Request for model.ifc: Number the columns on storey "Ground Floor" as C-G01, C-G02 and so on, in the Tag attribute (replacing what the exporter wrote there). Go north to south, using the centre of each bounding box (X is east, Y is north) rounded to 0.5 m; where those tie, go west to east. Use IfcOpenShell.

First a look at what the model holds.

```python
import ifcopenshell
import ifcopenshell.util.element
import ifcopenshell.util.placement

model = ifcopenshell.open("model.ifc")
print(model.schema)
storey = next(s for s in model.by_type("IfcBuildingStorey") if s.Name == "Ground Floor")
columns = [e for e in ifcopenshell.util.element.get_decomposition(storey) if e.is_a("IfcColumn")]
for e in sorted(columns, key=lambda e: e.id()):
    origin = ifcopenshell.util.placement.get_local_placement(e.ObjectPlacement)[:3, 3]
    print(e.id(), e.Tag, e.Name, origin.round(2) + 0.0, sep=" | ")
```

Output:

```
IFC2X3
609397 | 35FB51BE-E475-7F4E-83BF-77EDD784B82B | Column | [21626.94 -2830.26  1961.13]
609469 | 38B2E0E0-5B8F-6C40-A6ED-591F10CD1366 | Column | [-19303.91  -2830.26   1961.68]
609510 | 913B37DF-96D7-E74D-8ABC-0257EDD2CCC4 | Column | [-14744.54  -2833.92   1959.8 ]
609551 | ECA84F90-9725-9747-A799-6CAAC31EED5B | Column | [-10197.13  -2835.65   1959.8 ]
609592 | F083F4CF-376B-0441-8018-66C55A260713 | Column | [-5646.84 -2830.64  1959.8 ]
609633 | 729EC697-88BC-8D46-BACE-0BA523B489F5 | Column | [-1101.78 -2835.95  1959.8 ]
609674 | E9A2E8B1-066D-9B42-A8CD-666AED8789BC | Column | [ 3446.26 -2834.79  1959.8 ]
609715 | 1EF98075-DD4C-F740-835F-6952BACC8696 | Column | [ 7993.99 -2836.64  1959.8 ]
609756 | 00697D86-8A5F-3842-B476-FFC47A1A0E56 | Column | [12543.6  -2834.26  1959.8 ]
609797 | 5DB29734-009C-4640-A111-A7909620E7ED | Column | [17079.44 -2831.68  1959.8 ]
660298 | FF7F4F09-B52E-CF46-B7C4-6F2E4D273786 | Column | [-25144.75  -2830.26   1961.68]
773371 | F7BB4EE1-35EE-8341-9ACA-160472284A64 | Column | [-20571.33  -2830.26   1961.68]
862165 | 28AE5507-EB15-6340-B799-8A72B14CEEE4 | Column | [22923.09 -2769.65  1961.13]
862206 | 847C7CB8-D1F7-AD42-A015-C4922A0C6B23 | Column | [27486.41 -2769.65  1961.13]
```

```python
import ifcopenshell
import ifcopenshell.geom
import ifcopenshell.util.element
import ifcopenshell.util.shape

model = ifcopenshell.open("model.ifc")
settings = ifcopenshell.geom.settings()
settings.set("use-world-coords", True)


def centre(element):
    shape = ifcopenshell.geom.create_shape(settings, element)
    return ifcopenshell.util.shape.get_bbox_centroid(shape.geometry)


storey = next(s for s in model.by_type("IfcBuildingStorey") if s.Name == "Ground Floor")
columns = [e for e in ifcopenshell.util.element.get_decomposition(storey) if e.is_a("IfcColumn")]

# Insertion points can sit at a corner or the storey origin, so sort by the geometry (in metres).
centres = {e: centre(e) for e in columns}
columns.sort(key=lambda e: (-round(centres[e][1] / 0.5), centres[e][0]))

for i, e in enumerate(columns, start=1):
    number = f"C-G{i:02d}"
    e.Tag = number
    print(e.id(), number)

model.write("model_v2.ifc")
```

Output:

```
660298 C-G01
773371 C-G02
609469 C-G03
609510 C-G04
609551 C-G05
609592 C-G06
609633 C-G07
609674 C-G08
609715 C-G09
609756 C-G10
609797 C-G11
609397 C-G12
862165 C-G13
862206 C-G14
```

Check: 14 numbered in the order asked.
